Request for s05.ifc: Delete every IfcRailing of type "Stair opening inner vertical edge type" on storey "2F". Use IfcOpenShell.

First a look at what the model holds.

```python
import ifcopenshell
import ifcopenshell.util.element

model = ifcopenshell.open("s05.ifc")
print(model.schema)
storey = next(s for s in model.by_type("IfcBuildingStorey") if s.Name == "2F")
railings = [e for e in ifcopenshell.util.element.get_decomposition(storey) if e.is_a("IfcRailing")]
seen = {}
for e in railings:
    element_type = ifcopenshell.util.element.get_type(e)
    name = element_type.Name if element_type not in (None, e) else None
    seen[name] = seen.get(name, 0) + 1
for name, count in sorted(seen.items(), key=str):
    print(count, "x", name)
```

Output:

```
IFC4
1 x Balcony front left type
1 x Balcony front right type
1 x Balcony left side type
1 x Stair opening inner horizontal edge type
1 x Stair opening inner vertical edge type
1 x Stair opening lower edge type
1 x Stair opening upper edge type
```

```python
import ifcopenshell
import ifcopenshell.api.root
import ifcopenshell.util.element

model = ifcopenshell.open("s05.ifc")

storey = next(s for s in model.by_type("IfcBuildingStorey") if s.Name == "2F")
railings = [e for e in ifcopenshell.util.element.get_decomposition(storey) if e.is_a("IfcRailing")]
targets = [e for e in railings if (t := ifcopenshell.util.element.get_type(e)) not in (None, e) and t.Name == "Stair opening inner vertical edge type"]

for e in targets:
    ifcopenshell.api.root.remove_product(model, product=e)
print(len(targets), "removed")

model.write("s05_rev.ifc")
```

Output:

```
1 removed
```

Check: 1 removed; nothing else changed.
